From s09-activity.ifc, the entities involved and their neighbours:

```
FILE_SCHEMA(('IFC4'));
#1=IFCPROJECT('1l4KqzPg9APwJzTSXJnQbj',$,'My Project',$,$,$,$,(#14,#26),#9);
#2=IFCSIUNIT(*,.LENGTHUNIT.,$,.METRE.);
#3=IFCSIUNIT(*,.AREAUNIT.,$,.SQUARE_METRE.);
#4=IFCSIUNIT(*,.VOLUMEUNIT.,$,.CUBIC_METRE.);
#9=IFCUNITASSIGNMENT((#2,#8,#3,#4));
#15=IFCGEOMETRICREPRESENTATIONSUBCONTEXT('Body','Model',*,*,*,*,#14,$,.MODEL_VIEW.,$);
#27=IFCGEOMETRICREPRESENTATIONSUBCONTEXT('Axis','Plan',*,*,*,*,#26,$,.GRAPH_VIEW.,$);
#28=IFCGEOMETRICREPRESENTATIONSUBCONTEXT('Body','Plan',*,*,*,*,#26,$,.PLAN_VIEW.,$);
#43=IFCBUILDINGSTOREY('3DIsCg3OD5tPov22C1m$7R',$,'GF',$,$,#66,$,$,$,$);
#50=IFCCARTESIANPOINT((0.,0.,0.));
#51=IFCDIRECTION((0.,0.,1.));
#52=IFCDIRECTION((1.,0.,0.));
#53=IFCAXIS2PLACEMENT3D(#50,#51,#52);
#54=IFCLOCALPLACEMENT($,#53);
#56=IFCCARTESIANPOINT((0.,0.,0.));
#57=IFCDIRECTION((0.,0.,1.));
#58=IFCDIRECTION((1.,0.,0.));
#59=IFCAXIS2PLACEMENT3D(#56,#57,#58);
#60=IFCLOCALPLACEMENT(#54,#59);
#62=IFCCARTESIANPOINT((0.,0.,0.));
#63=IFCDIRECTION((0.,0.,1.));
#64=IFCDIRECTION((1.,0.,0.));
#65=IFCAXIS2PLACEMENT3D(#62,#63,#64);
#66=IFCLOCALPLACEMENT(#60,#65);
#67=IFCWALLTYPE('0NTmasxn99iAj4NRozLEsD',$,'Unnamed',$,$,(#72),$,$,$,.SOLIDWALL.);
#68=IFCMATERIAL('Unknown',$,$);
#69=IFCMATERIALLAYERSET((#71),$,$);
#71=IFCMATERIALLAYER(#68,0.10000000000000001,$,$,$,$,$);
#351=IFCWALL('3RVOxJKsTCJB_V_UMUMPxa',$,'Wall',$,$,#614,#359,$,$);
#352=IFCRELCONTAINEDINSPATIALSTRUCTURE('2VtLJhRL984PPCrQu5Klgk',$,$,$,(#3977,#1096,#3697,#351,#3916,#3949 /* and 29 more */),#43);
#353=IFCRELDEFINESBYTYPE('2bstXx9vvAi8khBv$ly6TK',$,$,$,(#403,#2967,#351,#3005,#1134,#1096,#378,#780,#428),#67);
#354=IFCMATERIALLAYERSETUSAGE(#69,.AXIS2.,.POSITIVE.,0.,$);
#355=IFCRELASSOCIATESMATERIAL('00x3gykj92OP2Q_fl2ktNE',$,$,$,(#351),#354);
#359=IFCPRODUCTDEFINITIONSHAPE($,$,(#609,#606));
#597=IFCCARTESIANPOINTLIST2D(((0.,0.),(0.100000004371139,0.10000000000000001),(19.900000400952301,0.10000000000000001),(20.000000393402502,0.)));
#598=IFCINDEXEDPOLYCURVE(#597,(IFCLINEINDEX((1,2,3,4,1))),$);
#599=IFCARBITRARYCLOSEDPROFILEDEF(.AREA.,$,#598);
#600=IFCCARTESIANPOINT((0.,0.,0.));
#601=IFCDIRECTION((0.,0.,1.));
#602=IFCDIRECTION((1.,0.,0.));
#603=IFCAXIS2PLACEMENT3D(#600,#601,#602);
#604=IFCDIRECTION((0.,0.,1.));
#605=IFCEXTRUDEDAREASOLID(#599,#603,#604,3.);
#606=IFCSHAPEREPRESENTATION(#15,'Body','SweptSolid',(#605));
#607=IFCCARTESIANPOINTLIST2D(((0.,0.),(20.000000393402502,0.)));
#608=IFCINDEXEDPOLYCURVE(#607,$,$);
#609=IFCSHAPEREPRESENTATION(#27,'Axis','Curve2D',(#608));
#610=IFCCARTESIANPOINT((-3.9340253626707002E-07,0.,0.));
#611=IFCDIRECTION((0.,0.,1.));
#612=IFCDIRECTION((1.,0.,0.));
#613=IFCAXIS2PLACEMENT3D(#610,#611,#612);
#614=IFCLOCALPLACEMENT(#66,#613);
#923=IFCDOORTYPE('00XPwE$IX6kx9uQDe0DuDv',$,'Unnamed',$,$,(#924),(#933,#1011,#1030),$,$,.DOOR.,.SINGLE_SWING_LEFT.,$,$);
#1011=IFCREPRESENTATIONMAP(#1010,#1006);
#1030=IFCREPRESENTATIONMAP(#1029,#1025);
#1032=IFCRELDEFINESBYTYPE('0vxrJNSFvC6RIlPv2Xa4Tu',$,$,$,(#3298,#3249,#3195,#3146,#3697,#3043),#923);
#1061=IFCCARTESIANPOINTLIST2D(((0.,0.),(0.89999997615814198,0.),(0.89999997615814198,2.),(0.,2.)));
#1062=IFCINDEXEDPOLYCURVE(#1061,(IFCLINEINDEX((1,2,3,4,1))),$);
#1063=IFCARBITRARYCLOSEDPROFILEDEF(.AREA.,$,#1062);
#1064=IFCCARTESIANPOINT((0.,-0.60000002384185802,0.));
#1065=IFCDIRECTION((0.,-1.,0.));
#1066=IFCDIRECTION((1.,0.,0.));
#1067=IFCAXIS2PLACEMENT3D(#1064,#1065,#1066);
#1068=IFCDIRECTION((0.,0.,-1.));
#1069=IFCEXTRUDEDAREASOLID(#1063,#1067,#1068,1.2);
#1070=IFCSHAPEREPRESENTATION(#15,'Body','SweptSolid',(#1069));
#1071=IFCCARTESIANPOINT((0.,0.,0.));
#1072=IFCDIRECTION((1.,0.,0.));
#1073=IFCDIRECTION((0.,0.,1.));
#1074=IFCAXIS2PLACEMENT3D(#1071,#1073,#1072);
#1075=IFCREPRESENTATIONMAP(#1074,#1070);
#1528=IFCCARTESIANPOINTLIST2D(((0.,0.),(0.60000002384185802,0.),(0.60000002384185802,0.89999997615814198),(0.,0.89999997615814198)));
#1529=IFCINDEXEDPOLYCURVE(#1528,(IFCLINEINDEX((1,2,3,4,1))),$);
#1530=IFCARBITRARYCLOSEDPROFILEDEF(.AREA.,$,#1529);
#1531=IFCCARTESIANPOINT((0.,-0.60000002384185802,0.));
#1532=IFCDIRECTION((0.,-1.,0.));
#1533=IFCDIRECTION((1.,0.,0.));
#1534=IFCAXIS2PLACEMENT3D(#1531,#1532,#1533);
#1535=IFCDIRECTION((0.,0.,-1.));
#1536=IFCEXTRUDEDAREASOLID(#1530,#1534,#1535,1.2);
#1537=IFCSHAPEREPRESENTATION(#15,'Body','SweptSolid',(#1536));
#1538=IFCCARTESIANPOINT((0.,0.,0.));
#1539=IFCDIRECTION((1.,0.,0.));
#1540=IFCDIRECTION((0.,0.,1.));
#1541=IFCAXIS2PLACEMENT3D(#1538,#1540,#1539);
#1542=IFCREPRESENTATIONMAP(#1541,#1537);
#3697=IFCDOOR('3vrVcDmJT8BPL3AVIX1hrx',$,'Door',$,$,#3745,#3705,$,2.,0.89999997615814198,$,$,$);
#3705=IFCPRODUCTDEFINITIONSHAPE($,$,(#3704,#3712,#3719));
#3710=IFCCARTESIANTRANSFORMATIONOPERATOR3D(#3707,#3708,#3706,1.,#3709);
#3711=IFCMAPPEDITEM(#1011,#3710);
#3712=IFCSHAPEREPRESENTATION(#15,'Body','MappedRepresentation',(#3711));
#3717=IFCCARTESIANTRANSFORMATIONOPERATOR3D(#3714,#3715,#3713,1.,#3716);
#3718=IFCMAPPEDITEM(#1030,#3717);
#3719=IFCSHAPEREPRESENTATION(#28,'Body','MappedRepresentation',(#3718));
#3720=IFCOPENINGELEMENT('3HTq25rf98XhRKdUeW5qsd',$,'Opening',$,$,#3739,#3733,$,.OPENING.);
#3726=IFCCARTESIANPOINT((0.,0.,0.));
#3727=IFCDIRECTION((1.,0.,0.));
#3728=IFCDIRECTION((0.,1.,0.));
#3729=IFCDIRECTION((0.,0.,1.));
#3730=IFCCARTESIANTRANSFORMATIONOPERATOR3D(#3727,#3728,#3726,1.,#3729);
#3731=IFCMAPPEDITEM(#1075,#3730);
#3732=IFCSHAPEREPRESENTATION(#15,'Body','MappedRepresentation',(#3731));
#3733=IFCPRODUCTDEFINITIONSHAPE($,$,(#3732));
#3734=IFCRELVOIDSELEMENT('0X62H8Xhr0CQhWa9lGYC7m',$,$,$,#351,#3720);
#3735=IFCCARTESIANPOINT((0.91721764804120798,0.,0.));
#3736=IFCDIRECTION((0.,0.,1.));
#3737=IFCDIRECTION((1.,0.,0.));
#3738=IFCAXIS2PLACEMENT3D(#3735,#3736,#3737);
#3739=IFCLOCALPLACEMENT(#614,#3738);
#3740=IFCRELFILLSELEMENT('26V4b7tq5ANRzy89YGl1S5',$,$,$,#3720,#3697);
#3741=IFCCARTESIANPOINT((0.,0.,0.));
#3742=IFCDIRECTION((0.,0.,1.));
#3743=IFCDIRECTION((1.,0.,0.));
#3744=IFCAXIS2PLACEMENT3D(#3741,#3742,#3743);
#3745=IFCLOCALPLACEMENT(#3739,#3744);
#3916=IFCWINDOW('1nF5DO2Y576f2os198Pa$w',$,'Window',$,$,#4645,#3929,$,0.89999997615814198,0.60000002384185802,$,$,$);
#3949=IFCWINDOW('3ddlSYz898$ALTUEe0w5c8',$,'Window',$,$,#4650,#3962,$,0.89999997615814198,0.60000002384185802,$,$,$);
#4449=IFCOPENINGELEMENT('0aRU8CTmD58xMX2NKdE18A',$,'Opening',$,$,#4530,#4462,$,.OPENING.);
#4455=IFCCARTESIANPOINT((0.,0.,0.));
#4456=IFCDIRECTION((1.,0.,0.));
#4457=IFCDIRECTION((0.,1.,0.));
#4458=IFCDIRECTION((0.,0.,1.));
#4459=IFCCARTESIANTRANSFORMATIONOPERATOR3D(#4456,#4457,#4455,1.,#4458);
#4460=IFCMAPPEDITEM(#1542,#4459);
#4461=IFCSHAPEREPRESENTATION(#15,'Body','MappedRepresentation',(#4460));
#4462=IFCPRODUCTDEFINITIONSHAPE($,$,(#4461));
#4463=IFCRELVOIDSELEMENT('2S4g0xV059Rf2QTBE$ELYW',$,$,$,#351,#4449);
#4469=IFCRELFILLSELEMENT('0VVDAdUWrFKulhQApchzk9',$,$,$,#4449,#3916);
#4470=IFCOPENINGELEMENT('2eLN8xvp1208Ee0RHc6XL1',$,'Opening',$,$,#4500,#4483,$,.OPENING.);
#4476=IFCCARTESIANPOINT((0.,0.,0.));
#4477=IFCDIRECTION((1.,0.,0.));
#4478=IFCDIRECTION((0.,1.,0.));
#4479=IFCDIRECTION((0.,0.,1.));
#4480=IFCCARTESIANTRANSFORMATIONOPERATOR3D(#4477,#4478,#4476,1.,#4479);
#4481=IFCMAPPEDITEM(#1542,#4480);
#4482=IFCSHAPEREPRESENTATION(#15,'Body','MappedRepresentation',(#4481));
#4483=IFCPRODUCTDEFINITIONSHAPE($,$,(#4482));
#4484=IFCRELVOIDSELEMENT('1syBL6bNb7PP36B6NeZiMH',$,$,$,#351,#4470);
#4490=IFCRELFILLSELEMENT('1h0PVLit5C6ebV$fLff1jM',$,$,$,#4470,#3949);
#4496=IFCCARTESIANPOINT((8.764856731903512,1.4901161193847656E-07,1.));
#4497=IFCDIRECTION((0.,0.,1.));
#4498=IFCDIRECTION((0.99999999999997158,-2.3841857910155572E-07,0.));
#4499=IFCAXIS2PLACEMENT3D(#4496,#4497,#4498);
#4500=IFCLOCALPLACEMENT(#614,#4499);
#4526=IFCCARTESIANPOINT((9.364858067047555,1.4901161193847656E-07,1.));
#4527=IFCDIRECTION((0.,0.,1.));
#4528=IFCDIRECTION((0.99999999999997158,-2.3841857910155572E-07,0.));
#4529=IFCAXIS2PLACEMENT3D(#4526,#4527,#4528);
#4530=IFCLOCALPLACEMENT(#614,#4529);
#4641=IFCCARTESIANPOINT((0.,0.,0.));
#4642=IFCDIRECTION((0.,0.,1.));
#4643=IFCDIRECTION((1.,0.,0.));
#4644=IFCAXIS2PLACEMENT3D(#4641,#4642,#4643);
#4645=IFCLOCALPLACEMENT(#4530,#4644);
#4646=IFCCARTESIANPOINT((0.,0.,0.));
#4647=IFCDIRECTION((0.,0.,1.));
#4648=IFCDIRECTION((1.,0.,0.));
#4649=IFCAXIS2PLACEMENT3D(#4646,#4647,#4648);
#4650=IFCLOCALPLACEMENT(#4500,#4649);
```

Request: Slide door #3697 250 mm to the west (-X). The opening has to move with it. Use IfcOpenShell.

```python
import ifcopenshell
import ifcopenshell.api.geometry
import ifcopenshell.util.placement
import ifcopenshell.util.unit

model = ifcopenshell.open("s09-activity.ifc")
unit_scale = ifcopenshell.util.unit.calculate_unit_scale(model)

door = model.by_guid("3vrVcDmJT8BPL3AVIX1hrx")
opening = door.FillsVoids[0].RelatingOpeningElement
wall = opening.VoidsElements[0].RelatingBuildingElement

wall_matrix = ifcopenshell.util.placement.get_local_placement(wall.ObjectPlacement)
shift = wall_matrix[:3, 0] * -0.25 / unit_scale
before = ifcopenshell.util.placement.get_local_placement(door.ObjectPlacement)[:3, 3].copy()

# The door is placed relative to its opening, so it follows when the opening moves.
matrix = ifcopenshell.util.placement.get_local_placement(opening.ObjectPlacement)
matrix[:3, 3] += shift
ifcopenshell.api.geometry.edit_object_placement(
    model, product=opening, matrix=matrix, is_si=False, should_transform_children=True
)

after = ifcopenshell.util.placement.get_local_placement(door.ObjectPlacement)[:3, 3]
print("door moved by", (after - before).round(3) + 0.0)

model.write("s09-activity_rev.ifc")
```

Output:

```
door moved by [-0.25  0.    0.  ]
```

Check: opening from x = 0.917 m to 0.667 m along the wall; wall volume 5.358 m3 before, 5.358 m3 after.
